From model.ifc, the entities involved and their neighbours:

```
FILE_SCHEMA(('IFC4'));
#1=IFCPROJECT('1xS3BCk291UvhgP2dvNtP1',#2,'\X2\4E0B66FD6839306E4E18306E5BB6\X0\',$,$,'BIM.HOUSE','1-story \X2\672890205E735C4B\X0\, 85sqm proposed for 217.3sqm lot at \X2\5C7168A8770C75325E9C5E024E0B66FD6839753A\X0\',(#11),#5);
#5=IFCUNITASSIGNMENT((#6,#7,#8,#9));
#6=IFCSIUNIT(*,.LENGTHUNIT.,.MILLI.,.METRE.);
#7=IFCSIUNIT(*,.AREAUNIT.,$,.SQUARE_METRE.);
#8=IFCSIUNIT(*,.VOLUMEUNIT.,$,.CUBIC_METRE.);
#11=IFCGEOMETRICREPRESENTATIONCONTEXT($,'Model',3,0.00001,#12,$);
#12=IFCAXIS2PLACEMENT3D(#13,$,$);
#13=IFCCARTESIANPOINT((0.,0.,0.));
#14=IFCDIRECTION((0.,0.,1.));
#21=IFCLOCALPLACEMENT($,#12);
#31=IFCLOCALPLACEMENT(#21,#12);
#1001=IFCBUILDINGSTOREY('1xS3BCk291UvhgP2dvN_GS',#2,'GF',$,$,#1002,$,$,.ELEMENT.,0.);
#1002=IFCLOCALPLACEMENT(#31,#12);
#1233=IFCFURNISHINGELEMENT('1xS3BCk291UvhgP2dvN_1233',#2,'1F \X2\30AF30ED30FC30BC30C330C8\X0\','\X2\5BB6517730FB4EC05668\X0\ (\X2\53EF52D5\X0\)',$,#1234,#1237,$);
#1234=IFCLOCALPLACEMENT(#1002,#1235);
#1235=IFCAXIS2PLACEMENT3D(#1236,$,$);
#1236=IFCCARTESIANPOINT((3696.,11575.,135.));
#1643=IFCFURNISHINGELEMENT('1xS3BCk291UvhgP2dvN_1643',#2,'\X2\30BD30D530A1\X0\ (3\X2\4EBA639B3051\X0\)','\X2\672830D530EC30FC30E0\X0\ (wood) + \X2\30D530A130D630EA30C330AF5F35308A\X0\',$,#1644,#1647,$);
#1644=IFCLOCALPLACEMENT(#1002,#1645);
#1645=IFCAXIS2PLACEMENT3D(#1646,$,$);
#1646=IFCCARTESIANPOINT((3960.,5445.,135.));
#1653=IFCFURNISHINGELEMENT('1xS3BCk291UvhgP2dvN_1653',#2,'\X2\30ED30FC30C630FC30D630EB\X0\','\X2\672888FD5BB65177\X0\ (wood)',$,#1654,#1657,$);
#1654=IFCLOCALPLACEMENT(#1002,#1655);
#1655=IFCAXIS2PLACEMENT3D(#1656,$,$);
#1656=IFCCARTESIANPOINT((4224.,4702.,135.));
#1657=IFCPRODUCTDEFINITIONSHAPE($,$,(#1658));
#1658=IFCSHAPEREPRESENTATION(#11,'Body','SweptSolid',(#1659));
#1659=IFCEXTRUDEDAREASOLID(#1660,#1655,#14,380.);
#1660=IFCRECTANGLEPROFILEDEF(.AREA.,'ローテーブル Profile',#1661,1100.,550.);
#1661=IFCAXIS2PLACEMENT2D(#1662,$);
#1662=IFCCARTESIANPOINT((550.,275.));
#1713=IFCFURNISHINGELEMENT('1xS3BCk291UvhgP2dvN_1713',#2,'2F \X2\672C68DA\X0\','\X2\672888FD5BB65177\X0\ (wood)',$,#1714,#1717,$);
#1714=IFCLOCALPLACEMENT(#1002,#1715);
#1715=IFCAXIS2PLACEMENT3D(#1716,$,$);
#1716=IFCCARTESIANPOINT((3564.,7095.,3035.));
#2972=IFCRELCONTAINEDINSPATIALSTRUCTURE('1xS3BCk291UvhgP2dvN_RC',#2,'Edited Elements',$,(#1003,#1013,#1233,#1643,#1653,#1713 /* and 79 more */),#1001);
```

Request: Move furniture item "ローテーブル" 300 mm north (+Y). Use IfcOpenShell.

```python
import ifcopenshell
import ifcopenshell.api.geometry
import ifcopenshell.util.placement
import ifcopenshell.util.unit

model = ifcopenshell.open("model.ifc")
unit_scale = ifcopenshell.util.unit.calculate_unit_scale(model)

item = model.by_guid("1xS3BCk291UvhgP2dvN_1653")
matrix = ifcopenshell.util.placement.get_local_placement(item.ObjectPlacement)
matrix[1, 3] += 0.3 / unit_scale
ifcopenshell.api.geometry.edit_object_placement(model, product=item, matrix=matrix, is_si=False)

print(ifcopenshell.util.placement.get_local_placement(item.ObjectPlacement).round(3) + 0.0)

model.write("model-out.ifc")
```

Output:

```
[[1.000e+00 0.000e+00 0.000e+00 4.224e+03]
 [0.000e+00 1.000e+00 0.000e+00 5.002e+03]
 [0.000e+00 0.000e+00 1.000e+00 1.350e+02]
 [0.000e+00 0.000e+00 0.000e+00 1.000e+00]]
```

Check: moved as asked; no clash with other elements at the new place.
